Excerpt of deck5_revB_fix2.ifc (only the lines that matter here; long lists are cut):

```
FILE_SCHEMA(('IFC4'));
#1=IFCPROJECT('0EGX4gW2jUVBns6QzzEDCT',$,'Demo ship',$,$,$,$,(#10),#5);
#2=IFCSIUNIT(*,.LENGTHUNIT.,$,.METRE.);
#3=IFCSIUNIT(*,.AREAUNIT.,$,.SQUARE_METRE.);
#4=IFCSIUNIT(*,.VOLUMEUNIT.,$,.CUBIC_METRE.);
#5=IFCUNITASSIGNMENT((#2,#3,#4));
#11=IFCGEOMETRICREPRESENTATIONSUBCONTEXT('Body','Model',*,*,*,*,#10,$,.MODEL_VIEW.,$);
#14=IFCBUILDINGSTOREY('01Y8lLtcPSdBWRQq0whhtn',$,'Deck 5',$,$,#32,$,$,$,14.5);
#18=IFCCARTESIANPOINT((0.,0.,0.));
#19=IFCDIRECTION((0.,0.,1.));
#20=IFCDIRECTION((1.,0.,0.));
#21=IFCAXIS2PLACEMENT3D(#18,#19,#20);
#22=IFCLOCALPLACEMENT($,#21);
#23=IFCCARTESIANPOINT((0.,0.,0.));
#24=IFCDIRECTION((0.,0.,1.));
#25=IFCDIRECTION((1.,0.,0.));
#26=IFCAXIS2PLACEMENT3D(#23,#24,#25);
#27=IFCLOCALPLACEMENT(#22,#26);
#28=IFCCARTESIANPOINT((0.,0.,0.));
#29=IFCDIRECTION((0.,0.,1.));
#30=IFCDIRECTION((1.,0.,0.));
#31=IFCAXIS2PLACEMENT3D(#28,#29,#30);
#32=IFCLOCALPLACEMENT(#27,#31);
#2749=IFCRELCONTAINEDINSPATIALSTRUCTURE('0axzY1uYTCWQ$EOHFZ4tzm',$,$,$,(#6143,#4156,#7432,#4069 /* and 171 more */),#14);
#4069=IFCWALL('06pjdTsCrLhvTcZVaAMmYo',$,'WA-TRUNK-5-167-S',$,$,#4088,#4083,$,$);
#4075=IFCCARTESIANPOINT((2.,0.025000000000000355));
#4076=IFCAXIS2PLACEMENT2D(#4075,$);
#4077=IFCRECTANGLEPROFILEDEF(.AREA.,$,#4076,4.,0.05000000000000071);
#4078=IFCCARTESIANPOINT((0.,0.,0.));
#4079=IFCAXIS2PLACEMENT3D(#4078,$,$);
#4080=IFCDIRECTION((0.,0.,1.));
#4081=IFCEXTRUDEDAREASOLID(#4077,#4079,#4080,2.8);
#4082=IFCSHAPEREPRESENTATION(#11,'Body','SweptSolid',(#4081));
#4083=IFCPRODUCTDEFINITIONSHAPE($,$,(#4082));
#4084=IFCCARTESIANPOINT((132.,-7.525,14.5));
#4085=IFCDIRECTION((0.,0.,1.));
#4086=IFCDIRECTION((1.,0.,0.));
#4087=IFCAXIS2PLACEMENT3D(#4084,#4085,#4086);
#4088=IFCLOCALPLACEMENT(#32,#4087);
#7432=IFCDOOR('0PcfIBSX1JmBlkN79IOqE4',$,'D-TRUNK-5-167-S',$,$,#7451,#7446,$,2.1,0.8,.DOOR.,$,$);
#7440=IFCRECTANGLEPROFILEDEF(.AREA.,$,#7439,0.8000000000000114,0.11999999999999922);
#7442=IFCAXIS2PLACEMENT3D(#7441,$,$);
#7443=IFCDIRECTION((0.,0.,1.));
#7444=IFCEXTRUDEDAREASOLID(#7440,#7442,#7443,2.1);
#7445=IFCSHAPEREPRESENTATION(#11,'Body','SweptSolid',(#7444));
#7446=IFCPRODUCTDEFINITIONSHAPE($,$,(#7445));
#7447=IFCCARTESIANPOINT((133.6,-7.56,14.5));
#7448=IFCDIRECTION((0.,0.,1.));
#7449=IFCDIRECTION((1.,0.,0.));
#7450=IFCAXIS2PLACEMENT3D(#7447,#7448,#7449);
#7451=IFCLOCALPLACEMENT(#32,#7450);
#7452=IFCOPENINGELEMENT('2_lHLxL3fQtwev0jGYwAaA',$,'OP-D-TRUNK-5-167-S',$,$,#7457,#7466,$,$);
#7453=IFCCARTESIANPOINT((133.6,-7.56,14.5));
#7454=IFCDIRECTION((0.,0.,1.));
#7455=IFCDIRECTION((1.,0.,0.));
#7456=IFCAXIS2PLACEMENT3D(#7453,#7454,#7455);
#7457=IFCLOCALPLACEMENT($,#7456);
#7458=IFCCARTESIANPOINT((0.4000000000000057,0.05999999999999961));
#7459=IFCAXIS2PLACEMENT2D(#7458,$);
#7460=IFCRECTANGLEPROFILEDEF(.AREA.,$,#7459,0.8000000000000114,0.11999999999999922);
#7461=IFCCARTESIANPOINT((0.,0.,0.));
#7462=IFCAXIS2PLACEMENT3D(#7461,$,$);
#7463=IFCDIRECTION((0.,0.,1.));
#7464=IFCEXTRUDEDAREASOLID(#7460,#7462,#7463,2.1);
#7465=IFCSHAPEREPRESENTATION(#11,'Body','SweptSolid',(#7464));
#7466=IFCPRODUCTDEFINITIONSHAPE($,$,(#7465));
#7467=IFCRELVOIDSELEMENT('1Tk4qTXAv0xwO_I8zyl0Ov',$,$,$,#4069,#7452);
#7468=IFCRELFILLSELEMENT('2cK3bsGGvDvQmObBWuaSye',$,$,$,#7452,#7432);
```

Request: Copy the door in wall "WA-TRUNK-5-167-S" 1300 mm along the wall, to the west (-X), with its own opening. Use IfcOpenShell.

```python
import ifcopenshell
import ifcopenshell.api.feature
import ifcopenshell.api.geometry
import ifcopenshell.api.root
import ifcopenshell.geom
import ifcopenshell.util.element
import ifcopenshell.util.placement
import ifcopenshell.util.shape
import ifcopenshell.util.unit

model = ifcopenshell.open("deck5_revB_fix2.ifc")
unit_scale = ifcopenshell.util.unit.calculate_unit_scale(model)
settings = ifcopenshell.geom.settings()


def volume(element):
    """Net volume in cubic metres, openings subtracted."""
    shape = ifcopenshell.geom.create_shape(settings, element)
    return ifcopenshell.util.shape.get_volume(shape.geometry)


door = model.by_guid("0PcfIBSX1JmBlkN79IOqE4")
opening = door.FillsVoids[0].RelatingOpeningElement
wall = opening.VoidsElements[0].RelatingBuildingElement
before = volume(wall)
shift = ifcopenshell.util.placement.get_local_placement(wall.ObjectPlacement)[:3, 0] * -1.3 / unit_scale

# copy_class copies the void relationship, type, container and properties, but no geometry.
new_opening = ifcopenshell.api.root.copy_class(model, product=opening)
new_opening.Representation = ifcopenshell.util.element.copy_deep(
    model, opening.Representation, exclude=["IfcGeometricRepresentationContext", "IfcRepresentationMap"]
)
new_door = ifcopenshell.api.root.copy_class(model, product=door)
new_door.Representation = ifcopenshell.util.element.copy_deep(
    model, door.Representation, exclude=["IfcGeometricRepresentationContext", "IfcRepresentationMap"]
)
ifcopenshell.api.feature.add_filling(model, opening=new_opening, element=new_door)

for old, new in ((opening, new_opening), (door, new_door)):
    matrix = ifcopenshell.util.placement.get_local_placement(old.ObjectPlacement)
    matrix[:3, 3] += shift
    ifcopenshell.api.geometry.edit_object_placement(model, product=new, matrix=matrix, is_si=False)

after = volume(wall)

print(f"wall volume {before:.3f} -> {after:.3f} m3")

model.write("deck5_revB_fix2_edited.ifc")
```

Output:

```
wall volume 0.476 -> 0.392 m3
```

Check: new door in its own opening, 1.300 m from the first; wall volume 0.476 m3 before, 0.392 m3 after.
